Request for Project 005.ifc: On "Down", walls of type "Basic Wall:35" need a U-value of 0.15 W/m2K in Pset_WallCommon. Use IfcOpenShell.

First a look at what the model holds.

```python
import ifcopenshell
import ifcopenshell.util.element

model = ifcopenshell.open("Project 005.ifc")
print(model.schema)
storey = next(s for s in model.by_type("IfcBuildingStorey") if s.Name == "Down")
walls = [e for e in ifcopenshell.util.element.get_decomposition(storey) if e.is_a("IfcWall")]
seen = {}
for e in walls:
    element_type = ifcopenshell.util.element.get_type(e)
    key = (element_type.Name if element_type != e and element_type else None, ifcopenshell.util.element.get_pset(e, "Pset_WallCommon", "ThermalTransmittance"))
    seen[key] = seen.get(key, 0) + 1
for (name, value), count in sorted(seen.items(), key=str):
    print(count, "x", name, "|", value)
```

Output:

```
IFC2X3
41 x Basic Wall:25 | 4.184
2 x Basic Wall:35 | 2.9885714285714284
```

```python
import ifcopenshell
import ifcopenshell.api.pset
import ifcopenshell.util.element

model = ifcopenshell.open("Project 005.ifc")

storey = next(s for s in model.by_type("IfcBuildingStorey") if s.Name == "Down")
walls = [e for e in ifcopenshell.util.element.get_decomposition(storey) if e.is_a("IfcWall")]

count = 0
for e in walls:
    element_type = ifcopenshell.util.element.get_type(e)
    if element_type in (None, e) or element_type.Name != "Basic Wall:35":
        continue
    # add_pset returns the element's existing set when there is one.
    pset = ifcopenshell.api.pset.add_pset(model, product=e, name="Pset_WallCommon")
    ifcopenshell.api.pset.edit_pset(model, pset=pset, properties={"ThermalTransmittance": 0.15})
    count += 1

print(count, "walls updated")

model.write("Project 005-out.ifc")
```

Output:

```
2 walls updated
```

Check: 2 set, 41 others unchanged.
